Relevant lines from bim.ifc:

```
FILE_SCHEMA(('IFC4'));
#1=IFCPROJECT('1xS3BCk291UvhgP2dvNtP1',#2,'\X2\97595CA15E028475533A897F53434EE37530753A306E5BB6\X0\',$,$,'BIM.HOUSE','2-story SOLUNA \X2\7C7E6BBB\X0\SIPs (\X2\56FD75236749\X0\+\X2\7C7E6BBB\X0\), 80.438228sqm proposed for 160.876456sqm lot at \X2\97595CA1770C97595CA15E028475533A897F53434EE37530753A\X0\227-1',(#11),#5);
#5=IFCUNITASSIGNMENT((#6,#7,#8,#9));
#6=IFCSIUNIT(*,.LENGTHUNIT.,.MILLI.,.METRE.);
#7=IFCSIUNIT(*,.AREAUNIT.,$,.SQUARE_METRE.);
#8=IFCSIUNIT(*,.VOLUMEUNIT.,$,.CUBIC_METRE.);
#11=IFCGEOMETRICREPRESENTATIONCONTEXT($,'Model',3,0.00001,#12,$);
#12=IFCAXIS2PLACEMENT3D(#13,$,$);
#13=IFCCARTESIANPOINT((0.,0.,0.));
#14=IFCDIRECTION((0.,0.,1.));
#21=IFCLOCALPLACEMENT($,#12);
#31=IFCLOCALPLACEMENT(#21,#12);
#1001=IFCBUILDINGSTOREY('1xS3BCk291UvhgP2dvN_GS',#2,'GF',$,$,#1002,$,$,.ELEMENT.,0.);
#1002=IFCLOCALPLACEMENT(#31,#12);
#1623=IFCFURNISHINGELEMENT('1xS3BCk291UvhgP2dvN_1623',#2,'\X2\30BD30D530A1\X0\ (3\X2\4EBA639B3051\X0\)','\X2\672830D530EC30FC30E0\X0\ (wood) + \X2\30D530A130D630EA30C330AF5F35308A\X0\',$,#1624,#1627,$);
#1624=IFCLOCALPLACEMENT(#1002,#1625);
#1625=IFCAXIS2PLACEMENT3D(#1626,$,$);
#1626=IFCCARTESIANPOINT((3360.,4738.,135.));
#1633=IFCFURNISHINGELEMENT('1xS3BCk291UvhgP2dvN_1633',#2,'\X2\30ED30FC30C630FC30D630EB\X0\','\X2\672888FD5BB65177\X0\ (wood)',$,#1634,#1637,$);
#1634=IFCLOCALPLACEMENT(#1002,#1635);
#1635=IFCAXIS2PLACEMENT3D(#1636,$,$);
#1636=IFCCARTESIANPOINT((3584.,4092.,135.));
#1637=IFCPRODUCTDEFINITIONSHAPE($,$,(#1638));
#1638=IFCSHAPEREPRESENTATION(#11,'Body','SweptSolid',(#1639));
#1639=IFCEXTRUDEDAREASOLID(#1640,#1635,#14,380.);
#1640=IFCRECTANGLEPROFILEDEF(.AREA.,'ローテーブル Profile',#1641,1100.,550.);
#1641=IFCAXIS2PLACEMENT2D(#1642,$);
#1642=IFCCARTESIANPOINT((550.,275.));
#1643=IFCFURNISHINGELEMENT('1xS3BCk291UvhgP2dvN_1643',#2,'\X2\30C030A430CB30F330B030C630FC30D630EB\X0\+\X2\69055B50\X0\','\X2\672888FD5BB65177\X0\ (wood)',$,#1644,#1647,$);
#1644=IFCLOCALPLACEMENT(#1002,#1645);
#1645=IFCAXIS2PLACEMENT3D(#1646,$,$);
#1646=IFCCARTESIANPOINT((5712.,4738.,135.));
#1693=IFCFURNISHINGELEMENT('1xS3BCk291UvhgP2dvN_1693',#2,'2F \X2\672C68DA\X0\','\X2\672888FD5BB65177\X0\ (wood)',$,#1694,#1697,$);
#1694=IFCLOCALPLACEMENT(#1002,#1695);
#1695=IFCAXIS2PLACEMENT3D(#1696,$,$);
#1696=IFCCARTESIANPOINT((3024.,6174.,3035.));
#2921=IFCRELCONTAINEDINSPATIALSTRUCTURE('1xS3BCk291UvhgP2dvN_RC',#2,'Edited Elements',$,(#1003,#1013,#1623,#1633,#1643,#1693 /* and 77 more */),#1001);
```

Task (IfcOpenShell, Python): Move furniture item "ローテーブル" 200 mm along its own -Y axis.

```python
import ifcopenshell
import ifcopenshell.api.geometry
import ifcopenshell.util.placement
import ifcopenshell.util.unit

model = ifcopenshell.open("bim.ifc")
unit_scale = ifcopenshell.util.unit.calculate_unit_scale(model)

item = model.by_guid("1xS3BCk291UvhgP2dvN_1633")
matrix = ifcopenshell.util.placement.get_local_placement(item.ObjectPlacement)
matrix[:3, 3] -= matrix[:3, 1] * 0.2 / unit_scale
ifcopenshell.api.geometry.edit_object_placement(model, product=item, matrix=matrix, is_si=False)

print(ifcopenshell.util.placement.get_local_placement(item.ObjectPlacement).round(3) + 0.0)

model.write("bim_rev.ifc")
```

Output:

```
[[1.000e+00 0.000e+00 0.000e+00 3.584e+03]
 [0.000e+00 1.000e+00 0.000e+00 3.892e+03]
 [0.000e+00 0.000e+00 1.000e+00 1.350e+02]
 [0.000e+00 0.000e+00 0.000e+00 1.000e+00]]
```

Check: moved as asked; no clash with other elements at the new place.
